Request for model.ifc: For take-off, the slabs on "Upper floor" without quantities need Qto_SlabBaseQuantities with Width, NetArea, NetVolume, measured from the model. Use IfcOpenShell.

First a look at what the model holds.

```python
import ifcopenshell
import ifcopenshell.util.element
import ifcopenshell.util.unit

model = ifcopenshell.open("model.ifc")
print(model.schema)
for unit_type in ("LENGTHUNIT", "AREAUNIT", "VOLUMEUNIT"):
    print(unit_type, ifcopenshell.util.unit.calculate_unit_scale(model, unit_type))
storey = next(s for s in model.by_type("IfcBuildingStorey") if s.Name == "Upper floor")
slabs = [e for e in ifcopenshell.util.element.get_decomposition(storey) if e.is_a("IfcSlab")]
for e in sorted(slabs, key=lambda e: e.id()):
    print(e.id(), e.is_a(), e.Name, list(ifcopenshell.util.element.get_psets(e, qtos_only=True)), sep=" | ")
```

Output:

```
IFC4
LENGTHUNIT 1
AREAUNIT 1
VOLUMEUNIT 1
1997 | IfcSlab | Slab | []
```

```python
import ifcopenshell
import ifcopenshell.api.pset
import ifcopenshell.geom
import ifcopenshell.util.element
import ifcopenshell.util.shape
import ifcopenshell.util.unit

model = ifcopenshell.open("model.ifc")
unit_scale = ifcopenshell.util.unit.calculate_unit_scale(model)
area_scale = ifcopenshell.util.unit.calculate_unit_scale(model, "AREAUNIT")
volume_scale = ifcopenshell.util.unit.calculate_unit_scale(model, "VOLUMEUNIT")
settings = ifcopenshell.geom.settings()

storey = next(s for s in model.by_type("IfcBuildingStorey") if s.Name == "Upper floor")
slabs = [e for e in ifcopenshell.util.element.get_decomposition(storey) if e.is_a("IfcSlab")]

for e in sorted(slabs, key=lambda e: e.id()):
    if ifcopenshell.util.element.get_psets(e, qtos_only=True, should_inherit=False):
        continue
    # Geometry comes back in metres, in the element's own axes.
    shape = ifcopenshell.geom.create_shape(settings, e)
    values = {
        "Width": ifcopenshell.util.shape.get_z(shape.geometry) / unit_scale,
        "NetArea": ifcopenshell.util.shape.get_footprint_area(shape.geometry) / area_scale,
        "NetVolume": ifcopenshell.util.shape.get_volume(shape.geometry) / volume_scale,
    }
    qto = ifcopenshell.api.pset.add_qto(model, product=e, name="Qto_SlabBaseQuantities")
    ifcopenshell.api.pset.edit_qto(model, qto=qto, properties=values)
    print(e.id(), {k: round(v, 3) for k, v in values.items()})

model.write("model_rev.ifc")
```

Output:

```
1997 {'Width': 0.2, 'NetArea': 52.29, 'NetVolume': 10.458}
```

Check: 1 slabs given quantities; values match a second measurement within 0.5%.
